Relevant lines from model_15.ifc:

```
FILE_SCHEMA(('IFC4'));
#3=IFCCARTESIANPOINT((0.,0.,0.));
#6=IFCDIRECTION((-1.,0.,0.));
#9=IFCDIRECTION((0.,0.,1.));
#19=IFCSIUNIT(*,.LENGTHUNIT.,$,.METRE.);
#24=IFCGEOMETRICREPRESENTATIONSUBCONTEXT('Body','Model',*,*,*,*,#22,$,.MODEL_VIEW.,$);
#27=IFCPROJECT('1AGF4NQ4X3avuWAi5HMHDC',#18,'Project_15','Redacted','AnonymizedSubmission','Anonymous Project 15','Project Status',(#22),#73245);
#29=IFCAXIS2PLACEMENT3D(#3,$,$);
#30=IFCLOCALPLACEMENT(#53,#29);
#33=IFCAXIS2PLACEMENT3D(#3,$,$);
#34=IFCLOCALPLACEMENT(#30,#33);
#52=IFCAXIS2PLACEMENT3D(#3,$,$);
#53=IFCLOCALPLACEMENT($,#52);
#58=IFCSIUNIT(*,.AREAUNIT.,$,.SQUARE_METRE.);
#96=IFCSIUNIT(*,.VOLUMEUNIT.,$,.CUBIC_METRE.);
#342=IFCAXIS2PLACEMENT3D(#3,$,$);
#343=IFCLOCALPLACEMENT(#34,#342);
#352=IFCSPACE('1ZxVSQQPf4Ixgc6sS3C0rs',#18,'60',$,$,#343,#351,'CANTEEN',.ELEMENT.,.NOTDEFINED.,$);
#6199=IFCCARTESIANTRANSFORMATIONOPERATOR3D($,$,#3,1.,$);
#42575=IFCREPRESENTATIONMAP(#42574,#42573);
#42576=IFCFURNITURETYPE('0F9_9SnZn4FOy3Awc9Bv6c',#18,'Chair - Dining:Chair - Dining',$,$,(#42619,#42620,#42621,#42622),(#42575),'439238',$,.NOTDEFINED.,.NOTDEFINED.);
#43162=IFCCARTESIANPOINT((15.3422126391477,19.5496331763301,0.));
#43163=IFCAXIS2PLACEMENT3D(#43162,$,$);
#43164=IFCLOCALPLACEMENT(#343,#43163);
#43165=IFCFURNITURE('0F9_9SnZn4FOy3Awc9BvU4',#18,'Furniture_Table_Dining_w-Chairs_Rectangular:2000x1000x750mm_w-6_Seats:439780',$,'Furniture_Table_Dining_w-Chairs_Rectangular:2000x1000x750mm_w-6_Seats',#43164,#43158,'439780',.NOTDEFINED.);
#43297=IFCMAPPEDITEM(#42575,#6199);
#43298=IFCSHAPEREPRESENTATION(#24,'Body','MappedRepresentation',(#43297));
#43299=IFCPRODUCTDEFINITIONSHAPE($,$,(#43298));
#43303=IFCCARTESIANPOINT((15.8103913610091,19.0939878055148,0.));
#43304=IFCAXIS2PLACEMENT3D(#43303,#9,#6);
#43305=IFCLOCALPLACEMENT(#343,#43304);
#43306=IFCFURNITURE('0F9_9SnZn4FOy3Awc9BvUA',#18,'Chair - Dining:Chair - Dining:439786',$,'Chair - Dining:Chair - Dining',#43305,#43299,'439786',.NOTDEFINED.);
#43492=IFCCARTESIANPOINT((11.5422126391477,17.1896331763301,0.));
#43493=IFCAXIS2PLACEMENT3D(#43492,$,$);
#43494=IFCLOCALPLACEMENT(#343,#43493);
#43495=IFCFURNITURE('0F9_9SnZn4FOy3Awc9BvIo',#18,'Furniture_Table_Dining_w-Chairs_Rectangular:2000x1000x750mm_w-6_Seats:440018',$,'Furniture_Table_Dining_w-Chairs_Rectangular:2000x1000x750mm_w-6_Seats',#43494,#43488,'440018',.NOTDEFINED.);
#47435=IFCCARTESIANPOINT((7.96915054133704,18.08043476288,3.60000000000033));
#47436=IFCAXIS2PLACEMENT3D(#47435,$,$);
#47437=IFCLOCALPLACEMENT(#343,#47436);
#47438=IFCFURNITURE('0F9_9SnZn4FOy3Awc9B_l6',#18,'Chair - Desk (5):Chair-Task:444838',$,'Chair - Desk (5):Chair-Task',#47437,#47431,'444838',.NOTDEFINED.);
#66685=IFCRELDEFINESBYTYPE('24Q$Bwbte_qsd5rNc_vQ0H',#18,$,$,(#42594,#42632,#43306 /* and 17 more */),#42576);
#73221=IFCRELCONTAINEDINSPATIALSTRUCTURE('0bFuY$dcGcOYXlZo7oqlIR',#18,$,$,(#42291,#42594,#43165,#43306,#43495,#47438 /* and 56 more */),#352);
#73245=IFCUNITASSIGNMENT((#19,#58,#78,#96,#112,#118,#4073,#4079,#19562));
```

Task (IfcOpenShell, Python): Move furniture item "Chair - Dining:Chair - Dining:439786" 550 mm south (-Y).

```python
import ifcopenshell
import ifcopenshell.api.geometry
import ifcopenshell.util.placement

model = ifcopenshell.open("model_15.ifc")

item = model.by_guid("0F9_9SnZn4FOy3Awc9BvUA")
matrix = ifcopenshell.util.placement.get_local_placement(item.ObjectPlacement)
matrix[1, 3] -= 0.55
ifcopenshell.api.geometry.edit_object_placement(model, product=item, matrix=matrix, is_si=False)

print(ifcopenshell.util.placement.get_local_placement(item.ObjectPlacement).round(3) + 0.0)

model.write("model_15_updated.ifc")
```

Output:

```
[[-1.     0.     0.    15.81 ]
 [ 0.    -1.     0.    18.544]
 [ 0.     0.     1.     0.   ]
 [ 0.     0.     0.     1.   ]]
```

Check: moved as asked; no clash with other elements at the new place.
